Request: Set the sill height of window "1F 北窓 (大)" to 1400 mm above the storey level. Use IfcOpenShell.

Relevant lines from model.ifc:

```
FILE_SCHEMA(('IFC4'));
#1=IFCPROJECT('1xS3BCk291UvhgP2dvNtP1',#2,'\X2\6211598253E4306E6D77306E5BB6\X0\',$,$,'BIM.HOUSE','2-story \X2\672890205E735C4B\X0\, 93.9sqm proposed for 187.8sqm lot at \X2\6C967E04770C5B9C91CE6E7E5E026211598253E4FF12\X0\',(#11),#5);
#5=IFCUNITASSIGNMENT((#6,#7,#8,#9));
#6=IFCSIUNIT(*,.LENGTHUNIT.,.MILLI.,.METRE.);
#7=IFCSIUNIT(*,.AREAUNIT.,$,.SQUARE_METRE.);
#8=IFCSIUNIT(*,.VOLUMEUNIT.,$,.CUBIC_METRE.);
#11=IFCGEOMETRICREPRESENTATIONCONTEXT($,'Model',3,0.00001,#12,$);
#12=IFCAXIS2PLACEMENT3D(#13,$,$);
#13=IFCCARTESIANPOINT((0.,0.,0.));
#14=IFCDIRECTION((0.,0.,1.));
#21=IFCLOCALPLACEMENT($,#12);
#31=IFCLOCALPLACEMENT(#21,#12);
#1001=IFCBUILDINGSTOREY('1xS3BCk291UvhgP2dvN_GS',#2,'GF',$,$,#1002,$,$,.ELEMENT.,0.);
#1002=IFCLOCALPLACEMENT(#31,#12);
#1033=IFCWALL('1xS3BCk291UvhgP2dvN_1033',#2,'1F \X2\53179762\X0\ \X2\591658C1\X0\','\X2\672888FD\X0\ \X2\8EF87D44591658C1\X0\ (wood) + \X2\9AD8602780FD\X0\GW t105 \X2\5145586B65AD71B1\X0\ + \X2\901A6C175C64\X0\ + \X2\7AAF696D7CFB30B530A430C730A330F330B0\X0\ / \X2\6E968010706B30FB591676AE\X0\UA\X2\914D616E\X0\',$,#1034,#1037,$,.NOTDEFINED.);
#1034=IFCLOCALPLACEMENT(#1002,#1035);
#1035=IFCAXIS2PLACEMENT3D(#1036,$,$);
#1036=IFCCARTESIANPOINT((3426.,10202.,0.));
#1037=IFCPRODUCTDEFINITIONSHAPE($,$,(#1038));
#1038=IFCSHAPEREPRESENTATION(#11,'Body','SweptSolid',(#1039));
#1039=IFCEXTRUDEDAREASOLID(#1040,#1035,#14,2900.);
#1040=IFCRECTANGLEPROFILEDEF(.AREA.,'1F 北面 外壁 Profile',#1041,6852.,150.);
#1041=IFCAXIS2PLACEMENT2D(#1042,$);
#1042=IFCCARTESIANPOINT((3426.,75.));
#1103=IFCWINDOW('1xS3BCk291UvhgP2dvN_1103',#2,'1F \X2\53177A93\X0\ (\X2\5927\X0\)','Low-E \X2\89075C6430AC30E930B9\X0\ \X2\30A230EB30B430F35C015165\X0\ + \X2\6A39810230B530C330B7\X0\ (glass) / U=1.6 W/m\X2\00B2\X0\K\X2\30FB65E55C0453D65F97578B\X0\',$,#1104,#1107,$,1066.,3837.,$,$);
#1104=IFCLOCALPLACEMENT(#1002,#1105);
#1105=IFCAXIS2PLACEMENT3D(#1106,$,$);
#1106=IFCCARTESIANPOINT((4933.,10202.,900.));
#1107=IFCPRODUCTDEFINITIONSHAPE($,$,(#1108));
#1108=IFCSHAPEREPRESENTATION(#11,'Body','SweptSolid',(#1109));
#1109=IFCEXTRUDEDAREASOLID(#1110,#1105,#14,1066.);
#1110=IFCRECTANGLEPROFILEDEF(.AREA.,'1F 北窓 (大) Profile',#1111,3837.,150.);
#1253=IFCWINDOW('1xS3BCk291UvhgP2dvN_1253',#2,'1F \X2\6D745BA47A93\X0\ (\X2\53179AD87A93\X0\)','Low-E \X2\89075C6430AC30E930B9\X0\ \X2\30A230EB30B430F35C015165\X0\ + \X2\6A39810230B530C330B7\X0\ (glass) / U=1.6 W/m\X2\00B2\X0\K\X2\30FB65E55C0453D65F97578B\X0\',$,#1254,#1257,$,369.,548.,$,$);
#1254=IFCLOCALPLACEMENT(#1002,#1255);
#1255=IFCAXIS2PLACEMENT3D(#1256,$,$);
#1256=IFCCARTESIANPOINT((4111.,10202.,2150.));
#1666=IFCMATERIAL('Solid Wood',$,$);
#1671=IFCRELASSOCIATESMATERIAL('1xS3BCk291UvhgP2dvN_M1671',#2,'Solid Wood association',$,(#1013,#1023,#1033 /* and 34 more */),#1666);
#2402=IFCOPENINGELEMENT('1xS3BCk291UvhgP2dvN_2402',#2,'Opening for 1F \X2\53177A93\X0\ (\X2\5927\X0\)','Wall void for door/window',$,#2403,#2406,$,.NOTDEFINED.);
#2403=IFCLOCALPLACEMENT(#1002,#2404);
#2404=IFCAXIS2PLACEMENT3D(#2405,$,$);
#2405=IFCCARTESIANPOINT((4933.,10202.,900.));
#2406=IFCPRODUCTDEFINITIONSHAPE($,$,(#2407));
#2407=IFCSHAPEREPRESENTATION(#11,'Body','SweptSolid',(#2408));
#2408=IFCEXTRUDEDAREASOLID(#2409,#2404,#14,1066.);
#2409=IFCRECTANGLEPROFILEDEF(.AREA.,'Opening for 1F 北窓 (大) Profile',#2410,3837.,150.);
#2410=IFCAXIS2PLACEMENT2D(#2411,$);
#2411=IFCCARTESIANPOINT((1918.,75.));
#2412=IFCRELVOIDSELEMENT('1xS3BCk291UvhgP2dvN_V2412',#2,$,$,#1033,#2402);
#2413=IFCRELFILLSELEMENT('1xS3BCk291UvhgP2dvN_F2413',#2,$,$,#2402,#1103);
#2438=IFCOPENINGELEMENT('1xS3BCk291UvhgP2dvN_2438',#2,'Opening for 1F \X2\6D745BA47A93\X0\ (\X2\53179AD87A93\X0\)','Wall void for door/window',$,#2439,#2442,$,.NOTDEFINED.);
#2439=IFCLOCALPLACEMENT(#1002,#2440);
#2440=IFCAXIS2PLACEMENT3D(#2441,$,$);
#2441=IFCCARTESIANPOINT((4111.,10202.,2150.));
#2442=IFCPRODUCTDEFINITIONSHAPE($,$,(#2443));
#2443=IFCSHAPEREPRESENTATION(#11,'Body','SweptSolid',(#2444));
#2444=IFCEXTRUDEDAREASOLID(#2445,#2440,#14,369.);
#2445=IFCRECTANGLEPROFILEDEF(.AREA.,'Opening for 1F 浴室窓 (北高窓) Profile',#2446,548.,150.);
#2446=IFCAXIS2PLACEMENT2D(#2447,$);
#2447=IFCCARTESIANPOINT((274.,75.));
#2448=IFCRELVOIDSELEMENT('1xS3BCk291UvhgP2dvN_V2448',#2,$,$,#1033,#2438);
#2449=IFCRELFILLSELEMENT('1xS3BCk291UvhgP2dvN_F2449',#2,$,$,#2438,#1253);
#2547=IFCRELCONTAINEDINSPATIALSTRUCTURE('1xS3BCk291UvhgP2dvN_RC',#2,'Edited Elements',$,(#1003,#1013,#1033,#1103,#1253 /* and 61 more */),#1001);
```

```python
import numpy as np
import ifcopenshell
import ifcopenshell.api.geometry
import ifcopenshell.geom
import ifcopenshell.util.element
import ifcopenshell.util.placement
import ifcopenshell.util.shape
import ifcopenshell.util.unit

model = ifcopenshell.open("model.ifc")
unit_scale = ifcopenshell.util.unit.calculate_unit_scale(model)

window = model.by_guid("1xS3BCk291UvhgP2dvN_1103")
opening = window.FillsVoids[0].RelatingOpeningElement
storey = ifcopenshell.util.element.get_container(window, ifc_class="IfcBuildingStorey")
level = ifcopenshell.util.placement.get_local_placement(storey.ObjectPlacement)[2, 3]

# The opening's origin need not be at the sill, so measure its lowest point.
shape = ifcopenshell.geom.create_shape(ifcopenshell.geom.settings(), opening)
bottom = ifcopenshell.util.shape.get_shape_bottom_elevation(shape, shape.geometry) / unit_scale
dz = level + 1400.0 - bottom

shift = np.array([0.0, 0.0, dz])
# The window is not placed relative to its opening, so move both.
for product in (opening, window):
    matrix = ifcopenshell.util.placement.get_local_placement(product.ObjectPlacement)
    matrix[:3, 3] += shift
    ifcopenshell.api.geometry.edit_object_placement(model, product=product, matrix=matrix, is_si=False)

print(f"moved by {dz * unit_scale:+.3f} m")

model.write("model_v2.ifc")
```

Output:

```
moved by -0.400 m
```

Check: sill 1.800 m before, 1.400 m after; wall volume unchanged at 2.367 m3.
